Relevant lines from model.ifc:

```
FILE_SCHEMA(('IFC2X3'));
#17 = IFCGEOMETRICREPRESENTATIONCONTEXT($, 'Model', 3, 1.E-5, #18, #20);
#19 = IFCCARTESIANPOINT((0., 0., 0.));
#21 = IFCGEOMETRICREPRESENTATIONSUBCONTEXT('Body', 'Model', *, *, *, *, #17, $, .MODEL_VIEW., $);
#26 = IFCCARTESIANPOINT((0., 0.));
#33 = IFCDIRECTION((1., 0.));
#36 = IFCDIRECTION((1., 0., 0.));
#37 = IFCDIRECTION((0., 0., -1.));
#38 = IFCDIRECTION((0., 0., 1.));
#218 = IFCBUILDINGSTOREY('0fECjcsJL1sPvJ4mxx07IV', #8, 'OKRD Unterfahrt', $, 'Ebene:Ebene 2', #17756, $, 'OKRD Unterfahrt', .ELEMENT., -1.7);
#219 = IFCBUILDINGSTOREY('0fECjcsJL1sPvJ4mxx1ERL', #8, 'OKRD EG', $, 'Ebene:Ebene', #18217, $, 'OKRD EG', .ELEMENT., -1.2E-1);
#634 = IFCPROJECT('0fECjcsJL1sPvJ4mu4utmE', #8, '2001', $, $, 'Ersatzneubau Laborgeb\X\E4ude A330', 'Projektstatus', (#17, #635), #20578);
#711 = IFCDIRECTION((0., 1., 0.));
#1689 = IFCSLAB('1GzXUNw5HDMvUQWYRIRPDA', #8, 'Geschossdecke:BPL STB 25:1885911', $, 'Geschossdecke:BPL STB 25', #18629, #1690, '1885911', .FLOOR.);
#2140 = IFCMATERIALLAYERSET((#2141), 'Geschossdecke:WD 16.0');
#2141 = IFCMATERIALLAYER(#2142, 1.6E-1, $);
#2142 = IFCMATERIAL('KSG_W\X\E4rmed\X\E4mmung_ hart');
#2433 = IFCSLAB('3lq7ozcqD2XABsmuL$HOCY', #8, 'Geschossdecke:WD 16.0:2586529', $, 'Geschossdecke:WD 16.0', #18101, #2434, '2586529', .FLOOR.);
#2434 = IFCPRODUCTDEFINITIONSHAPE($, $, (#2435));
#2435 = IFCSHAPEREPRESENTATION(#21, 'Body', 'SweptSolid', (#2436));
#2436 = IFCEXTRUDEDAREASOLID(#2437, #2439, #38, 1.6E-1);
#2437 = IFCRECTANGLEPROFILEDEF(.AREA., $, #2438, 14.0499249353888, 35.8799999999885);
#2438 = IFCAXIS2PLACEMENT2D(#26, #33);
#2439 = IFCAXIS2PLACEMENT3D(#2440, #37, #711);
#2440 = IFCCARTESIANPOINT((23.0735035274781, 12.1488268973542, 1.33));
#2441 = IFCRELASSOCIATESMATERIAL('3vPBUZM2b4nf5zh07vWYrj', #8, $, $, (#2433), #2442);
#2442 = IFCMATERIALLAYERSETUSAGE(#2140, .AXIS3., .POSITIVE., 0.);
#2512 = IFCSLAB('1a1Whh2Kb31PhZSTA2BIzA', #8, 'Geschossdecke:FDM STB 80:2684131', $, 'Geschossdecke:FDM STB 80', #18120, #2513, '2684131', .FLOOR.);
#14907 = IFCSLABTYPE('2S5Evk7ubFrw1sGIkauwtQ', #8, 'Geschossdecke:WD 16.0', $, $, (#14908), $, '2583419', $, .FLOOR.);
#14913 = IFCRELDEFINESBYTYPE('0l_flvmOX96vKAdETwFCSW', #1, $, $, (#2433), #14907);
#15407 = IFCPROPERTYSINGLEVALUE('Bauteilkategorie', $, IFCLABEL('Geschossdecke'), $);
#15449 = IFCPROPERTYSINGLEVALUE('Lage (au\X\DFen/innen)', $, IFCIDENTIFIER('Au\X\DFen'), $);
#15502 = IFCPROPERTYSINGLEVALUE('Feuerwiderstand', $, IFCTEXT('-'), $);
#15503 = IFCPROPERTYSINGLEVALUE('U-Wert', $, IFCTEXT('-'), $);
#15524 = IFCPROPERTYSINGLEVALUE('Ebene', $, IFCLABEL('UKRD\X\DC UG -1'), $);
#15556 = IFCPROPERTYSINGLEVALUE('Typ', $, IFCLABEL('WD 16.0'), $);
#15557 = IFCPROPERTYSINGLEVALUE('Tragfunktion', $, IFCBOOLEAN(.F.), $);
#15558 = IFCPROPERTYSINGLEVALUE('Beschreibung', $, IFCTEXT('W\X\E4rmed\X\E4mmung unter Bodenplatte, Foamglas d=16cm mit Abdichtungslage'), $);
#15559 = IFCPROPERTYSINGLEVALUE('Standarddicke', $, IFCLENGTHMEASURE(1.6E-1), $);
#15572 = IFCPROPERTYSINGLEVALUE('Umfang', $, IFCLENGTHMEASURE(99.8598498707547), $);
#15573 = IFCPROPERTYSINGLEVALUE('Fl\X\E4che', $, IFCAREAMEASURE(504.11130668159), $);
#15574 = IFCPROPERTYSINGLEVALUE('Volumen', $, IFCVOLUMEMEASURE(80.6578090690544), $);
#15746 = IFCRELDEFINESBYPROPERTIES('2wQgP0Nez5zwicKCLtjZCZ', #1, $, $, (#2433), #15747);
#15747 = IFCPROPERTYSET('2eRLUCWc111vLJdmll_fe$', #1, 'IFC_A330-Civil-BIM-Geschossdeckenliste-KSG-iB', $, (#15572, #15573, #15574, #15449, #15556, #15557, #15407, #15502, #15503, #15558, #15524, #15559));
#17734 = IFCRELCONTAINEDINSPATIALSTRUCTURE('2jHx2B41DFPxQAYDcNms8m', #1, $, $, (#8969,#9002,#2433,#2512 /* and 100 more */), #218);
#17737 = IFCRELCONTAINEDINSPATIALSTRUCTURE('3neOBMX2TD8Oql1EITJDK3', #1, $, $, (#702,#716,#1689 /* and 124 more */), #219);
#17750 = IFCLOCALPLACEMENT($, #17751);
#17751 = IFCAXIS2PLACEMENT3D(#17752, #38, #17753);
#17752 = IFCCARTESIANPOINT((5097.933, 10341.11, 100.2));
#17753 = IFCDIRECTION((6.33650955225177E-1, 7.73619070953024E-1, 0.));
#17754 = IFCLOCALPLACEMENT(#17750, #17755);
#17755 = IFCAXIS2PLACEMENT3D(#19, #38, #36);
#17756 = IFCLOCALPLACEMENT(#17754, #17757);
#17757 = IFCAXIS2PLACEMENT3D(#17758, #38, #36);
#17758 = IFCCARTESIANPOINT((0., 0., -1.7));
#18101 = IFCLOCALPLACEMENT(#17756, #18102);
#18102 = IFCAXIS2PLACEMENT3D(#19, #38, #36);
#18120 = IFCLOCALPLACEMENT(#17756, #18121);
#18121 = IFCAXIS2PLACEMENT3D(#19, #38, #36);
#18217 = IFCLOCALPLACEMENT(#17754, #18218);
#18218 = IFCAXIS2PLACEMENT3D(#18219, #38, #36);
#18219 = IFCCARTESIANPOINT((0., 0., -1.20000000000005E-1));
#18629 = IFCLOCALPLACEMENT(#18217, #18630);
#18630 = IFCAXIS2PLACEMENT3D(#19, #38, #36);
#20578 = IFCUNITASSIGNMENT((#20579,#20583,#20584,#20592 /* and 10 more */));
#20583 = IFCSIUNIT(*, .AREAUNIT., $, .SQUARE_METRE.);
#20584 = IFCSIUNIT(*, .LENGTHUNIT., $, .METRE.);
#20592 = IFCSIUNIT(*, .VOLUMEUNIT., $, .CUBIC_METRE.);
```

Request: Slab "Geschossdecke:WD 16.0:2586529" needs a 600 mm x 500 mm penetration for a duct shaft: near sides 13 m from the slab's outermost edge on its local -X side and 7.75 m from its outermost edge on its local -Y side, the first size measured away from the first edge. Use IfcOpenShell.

```python
import numpy as np
import ifcopenshell
import ifcopenshell.api.feature
import ifcopenshell.api.geometry
import ifcopenshell.api.pset
import ifcopenshell.api.root
import ifcopenshell.geom
import ifcopenshell.util.element
import ifcopenshell.util.placement
import ifcopenshell.util.representation
import ifcopenshell.util.shape
import ifcopenshell.util.unit

model = ifcopenshell.open("model.ifc")
unit_scale = ifcopenshell.util.unit.calculate_unit_scale(model)
area_scale = ifcopenshell.util.unit.calculate_unit_scale(model, "AREAUNIT")
volume_scale = ifcopenshell.util.unit.calculate_unit_scale(model, "VOLUMEUNIT")
settings = ifcopenshell.geom.settings()


def volume(element):
    """Net volume in cubic metres, openings subtracted."""
    shape = ifcopenshell.geom.create_shape(settings, element)
    return ifcopenshell.util.shape.get_volume(shape.geometry)


slab = model.by_guid("3lq7ozcqD2XABsmuL$HOCY")
before = volume(slab)

# Extent in the slab's own axes, in metres. The edges named are its -X and -Y sides.
slab_shape = ifcopenshell.geom.create_shape(settings, slab)
vertices = ifcopenshell.util.shape.get_vertices(slab_shape.geometry)
x_min, y_min, bottom = vertices.min(axis=0)
top = vertices[:, 2].max()

opening = ifcopenshell.api.root.create_entity(model, ifc_class="IfcOpeningElement", name="Duct shaft opening")
context = ifcopenshell.util.representation.get_context(model, "Model", "Body", "MODEL_VIEW")
width, depth = 0.6, 0.5
outline = [(0.0, 0.0), (width, 0.0), (width, depth), (0.0, depth), (0.0, 0.0)]
# Overshoot both faces by 50 mm so the cut is clean.
shape = ifcopenshell.api.geometry.add_slab_representation(
    model, context=context, depth=top - bottom + 0.1, polyline=outline
)
ifcopenshell.api.geometry.assign_representation(model, product=opening, representation=shape)

matrix = ifcopenshell.util.placement.get_local_placement(slab.ObjectPlacement)
matrix[:, 3] = matrix @ np.append(np.array([x_min + 13, y_min + 7.75, bottom - 0.05]) / unit_scale, 1.0)
ifcopenshell.api.geometry.edit_object_placement(model, product=opening, matrix=matrix, is_si=False)
ifcopenshell.api.feature.add_feature(model, feature=opening, element=slab)

after = volume(slab)

# Update the slab's stored quantities.
pset = model.by_id(ifcopenshell.util.element.get_pset(slab, "IFC_A330-Civil-BIM-Geschossdeckenliste-KSG-iB", should_inherit=False)["id"])
ifcopenshell.api.pset.edit_pset(model, pset=pset, properties={
    "Fläche": model.create_entity("IfcAreaMeasure", after / (top - bottom) / area_scale),
    "Volumen": model.create_entity("IfcVolumeMeasure", after / volume_scale),
})

print(f"slab volume {before:.3f} -> {after:.3f} m3")

model.write("model_updated.ifc")
```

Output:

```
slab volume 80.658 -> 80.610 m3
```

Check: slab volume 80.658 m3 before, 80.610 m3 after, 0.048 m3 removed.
